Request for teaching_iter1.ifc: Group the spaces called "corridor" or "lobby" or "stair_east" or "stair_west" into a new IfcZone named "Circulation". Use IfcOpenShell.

First a look at what the model holds.

```python
import ifcopenshell

model = ifcopenshell.open("teaching_iter1.ifc")
print(model.schema)
seen = {}
for space in model.by_type("IfcSpace"):
    seen[space.LongName] = seen.get(space.LongName, 0) + 1
for name, count in sorted(seen.items(), key=str):
    print(count, "x", name)
print("zones:", [z.Name for z in model.by_type("IfcZone")][:20])
```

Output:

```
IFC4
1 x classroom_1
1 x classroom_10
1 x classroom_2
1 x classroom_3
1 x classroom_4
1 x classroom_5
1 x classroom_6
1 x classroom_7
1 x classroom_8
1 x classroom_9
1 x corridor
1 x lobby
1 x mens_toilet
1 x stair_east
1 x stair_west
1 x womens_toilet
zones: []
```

```python
import ifcopenshell
import ifcopenshell.api.group
import ifcopenshell.api.root

model = ifcopenshell.open("teaching_iter1.ifc")

names = {"corridor", "lobby", "stair_east", "stair_west"}
spaces = [s for s in model.by_type("IfcSpace") if s.LongName in names]

zone = ifcopenshell.api.root.create_entity(model, ifc_class="IfcZone", name="Circulation")
ifcopenshell.api.group.assign_group(model, products=spaces, group=zone)
print(len(spaces), "spaces in", zone.Name)

model.write("teaching_iter1_v2.ifc")
```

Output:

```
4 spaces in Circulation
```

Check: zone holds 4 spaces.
